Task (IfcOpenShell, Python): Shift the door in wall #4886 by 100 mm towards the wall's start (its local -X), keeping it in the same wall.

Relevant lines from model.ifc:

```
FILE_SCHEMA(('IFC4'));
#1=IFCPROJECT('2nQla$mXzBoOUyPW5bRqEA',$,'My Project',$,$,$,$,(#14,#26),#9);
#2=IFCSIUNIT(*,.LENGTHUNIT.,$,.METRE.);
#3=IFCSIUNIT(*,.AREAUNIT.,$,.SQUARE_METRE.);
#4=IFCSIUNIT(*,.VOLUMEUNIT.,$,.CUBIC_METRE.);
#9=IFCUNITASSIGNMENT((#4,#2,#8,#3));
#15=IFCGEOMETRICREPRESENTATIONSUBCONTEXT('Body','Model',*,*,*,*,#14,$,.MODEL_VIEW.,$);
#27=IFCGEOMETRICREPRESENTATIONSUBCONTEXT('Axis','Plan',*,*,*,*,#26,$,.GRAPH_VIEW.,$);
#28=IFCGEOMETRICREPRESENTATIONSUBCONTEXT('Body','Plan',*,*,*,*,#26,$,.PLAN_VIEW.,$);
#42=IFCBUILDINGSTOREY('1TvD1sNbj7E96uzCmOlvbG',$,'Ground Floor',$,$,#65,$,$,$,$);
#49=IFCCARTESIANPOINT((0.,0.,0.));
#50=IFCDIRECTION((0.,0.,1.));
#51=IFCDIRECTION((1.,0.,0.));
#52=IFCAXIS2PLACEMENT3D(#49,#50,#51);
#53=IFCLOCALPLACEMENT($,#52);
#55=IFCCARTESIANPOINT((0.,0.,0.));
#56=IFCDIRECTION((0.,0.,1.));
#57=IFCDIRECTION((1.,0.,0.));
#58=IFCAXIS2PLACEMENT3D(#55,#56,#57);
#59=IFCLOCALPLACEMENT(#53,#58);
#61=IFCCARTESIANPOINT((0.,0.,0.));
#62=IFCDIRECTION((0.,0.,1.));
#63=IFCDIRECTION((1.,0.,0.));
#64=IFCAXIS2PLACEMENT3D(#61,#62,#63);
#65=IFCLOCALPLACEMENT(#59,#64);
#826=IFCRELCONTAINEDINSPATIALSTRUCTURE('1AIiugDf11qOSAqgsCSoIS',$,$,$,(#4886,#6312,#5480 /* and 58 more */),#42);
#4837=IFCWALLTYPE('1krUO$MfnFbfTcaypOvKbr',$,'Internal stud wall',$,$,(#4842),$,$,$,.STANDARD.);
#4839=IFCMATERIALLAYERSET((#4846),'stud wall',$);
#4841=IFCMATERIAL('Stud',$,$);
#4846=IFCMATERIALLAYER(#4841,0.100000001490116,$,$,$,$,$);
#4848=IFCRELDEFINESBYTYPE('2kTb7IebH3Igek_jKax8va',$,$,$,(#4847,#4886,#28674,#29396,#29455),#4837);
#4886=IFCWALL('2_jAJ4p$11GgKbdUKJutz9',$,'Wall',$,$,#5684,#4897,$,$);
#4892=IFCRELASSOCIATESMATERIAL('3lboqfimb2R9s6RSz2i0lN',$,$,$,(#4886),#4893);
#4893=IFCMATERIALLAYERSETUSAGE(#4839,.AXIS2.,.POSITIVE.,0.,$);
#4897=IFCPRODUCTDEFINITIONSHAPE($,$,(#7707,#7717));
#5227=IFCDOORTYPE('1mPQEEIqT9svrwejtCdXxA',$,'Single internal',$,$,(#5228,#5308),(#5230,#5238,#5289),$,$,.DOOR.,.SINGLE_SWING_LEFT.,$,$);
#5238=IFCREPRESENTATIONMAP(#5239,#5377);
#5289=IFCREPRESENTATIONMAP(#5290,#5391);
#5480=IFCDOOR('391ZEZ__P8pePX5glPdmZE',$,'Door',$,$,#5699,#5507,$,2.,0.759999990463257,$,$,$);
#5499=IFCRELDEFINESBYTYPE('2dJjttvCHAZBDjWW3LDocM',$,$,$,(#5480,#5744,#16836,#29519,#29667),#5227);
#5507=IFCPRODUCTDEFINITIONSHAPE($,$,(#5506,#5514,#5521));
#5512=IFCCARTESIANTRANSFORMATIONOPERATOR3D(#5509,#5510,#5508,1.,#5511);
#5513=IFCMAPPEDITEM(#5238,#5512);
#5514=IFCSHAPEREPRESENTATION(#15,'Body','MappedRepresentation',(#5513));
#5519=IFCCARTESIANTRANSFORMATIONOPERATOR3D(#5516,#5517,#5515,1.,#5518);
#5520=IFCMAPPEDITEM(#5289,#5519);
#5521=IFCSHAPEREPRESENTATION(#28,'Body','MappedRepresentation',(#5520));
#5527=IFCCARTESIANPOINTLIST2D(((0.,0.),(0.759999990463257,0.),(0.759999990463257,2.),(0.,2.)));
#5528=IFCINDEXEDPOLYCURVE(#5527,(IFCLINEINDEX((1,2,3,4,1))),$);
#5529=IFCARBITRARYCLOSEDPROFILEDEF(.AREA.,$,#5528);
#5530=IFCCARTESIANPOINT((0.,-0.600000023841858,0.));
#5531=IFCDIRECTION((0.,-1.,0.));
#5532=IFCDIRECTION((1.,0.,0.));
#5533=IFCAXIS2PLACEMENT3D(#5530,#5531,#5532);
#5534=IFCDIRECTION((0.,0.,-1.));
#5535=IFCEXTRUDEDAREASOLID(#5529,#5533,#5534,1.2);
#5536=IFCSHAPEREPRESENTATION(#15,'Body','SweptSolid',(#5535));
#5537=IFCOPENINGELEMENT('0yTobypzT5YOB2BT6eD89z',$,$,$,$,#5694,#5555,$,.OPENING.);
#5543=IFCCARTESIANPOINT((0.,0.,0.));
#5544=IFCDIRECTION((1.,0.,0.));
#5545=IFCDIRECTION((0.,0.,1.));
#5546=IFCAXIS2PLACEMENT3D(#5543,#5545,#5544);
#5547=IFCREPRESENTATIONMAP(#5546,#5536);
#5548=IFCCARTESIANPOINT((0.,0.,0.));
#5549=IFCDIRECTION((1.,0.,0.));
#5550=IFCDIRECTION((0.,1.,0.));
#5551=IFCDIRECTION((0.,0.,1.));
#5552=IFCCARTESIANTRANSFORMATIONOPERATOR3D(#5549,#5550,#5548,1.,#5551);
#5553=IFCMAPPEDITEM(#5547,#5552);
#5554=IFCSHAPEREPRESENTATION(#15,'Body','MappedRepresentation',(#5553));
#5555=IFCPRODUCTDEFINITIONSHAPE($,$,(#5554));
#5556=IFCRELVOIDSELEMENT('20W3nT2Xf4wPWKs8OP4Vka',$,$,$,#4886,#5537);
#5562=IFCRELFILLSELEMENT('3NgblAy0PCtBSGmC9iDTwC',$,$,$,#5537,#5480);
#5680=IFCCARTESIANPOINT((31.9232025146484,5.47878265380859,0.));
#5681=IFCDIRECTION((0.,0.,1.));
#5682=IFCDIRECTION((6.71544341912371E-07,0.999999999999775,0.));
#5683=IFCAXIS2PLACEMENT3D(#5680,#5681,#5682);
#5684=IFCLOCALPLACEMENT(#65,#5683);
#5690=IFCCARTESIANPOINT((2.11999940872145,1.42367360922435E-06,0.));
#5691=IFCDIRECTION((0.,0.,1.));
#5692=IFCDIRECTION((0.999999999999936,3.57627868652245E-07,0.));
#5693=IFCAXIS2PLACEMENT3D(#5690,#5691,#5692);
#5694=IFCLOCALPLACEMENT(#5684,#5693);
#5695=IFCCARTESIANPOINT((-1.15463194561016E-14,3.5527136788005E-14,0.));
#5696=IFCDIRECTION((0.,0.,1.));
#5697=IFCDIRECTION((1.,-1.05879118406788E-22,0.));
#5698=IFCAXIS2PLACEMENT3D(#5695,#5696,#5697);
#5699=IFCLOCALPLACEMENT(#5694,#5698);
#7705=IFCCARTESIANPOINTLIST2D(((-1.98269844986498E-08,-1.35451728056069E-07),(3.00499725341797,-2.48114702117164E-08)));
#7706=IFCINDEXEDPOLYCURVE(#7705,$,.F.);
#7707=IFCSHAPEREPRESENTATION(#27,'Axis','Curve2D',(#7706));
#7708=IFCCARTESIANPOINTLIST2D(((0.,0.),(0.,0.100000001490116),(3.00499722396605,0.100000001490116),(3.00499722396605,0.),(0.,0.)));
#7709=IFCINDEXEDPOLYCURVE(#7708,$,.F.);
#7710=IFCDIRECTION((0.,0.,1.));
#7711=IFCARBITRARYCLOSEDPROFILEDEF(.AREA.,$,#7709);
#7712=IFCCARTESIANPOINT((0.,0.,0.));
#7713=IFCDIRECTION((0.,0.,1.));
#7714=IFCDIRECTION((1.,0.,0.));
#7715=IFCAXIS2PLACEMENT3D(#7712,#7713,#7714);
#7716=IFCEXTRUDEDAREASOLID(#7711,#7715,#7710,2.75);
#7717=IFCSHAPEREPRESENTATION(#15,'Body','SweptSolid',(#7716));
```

```python
import ifcopenshell
import ifcopenshell.api.geometry
import ifcopenshell.util.placement
import ifcopenshell.util.unit

model = ifcopenshell.open("model.ifc")
unit_scale = ifcopenshell.util.unit.calculate_unit_scale(model)

door = model.by_guid("391ZEZ__P8pePX5glPdmZE")
opening = door.FillsVoids[0].RelatingOpeningElement
wall = opening.VoidsElements[0].RelatingBuildingElement

wall_matrix = ifcopenshell.util.placement.get_local_placement(wall.ObjectPlacement)
shift = wall_matrix[:3, 0] * -0.1 / unit_scale
before = ifcopenshell.util.placement.get_local_placement(door.ObjectPlacement)[:3, 3].copy()

# The door is placed relative to its opening, so it follows when the opening moves.
matrix = ifcopenshell.util.placement.get_local_placement(opening.ObjectPlacement)
matrix[:3, 3] += shift
ifcopenshell.api.geometry.edit_object_placement(
    model, product=opening, matrix=matrix, is_si=False, should_transform_children=True
)

after = ifcopenshell.util.placement.get_local_placement(door.ObjectPlacement)[:3, 3]
print("door moved by", (after - before).round(3) + 0.0)

model.write("model_updated.ifc")
```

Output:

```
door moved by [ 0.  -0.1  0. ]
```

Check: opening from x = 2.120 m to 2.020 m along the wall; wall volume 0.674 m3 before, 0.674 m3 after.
